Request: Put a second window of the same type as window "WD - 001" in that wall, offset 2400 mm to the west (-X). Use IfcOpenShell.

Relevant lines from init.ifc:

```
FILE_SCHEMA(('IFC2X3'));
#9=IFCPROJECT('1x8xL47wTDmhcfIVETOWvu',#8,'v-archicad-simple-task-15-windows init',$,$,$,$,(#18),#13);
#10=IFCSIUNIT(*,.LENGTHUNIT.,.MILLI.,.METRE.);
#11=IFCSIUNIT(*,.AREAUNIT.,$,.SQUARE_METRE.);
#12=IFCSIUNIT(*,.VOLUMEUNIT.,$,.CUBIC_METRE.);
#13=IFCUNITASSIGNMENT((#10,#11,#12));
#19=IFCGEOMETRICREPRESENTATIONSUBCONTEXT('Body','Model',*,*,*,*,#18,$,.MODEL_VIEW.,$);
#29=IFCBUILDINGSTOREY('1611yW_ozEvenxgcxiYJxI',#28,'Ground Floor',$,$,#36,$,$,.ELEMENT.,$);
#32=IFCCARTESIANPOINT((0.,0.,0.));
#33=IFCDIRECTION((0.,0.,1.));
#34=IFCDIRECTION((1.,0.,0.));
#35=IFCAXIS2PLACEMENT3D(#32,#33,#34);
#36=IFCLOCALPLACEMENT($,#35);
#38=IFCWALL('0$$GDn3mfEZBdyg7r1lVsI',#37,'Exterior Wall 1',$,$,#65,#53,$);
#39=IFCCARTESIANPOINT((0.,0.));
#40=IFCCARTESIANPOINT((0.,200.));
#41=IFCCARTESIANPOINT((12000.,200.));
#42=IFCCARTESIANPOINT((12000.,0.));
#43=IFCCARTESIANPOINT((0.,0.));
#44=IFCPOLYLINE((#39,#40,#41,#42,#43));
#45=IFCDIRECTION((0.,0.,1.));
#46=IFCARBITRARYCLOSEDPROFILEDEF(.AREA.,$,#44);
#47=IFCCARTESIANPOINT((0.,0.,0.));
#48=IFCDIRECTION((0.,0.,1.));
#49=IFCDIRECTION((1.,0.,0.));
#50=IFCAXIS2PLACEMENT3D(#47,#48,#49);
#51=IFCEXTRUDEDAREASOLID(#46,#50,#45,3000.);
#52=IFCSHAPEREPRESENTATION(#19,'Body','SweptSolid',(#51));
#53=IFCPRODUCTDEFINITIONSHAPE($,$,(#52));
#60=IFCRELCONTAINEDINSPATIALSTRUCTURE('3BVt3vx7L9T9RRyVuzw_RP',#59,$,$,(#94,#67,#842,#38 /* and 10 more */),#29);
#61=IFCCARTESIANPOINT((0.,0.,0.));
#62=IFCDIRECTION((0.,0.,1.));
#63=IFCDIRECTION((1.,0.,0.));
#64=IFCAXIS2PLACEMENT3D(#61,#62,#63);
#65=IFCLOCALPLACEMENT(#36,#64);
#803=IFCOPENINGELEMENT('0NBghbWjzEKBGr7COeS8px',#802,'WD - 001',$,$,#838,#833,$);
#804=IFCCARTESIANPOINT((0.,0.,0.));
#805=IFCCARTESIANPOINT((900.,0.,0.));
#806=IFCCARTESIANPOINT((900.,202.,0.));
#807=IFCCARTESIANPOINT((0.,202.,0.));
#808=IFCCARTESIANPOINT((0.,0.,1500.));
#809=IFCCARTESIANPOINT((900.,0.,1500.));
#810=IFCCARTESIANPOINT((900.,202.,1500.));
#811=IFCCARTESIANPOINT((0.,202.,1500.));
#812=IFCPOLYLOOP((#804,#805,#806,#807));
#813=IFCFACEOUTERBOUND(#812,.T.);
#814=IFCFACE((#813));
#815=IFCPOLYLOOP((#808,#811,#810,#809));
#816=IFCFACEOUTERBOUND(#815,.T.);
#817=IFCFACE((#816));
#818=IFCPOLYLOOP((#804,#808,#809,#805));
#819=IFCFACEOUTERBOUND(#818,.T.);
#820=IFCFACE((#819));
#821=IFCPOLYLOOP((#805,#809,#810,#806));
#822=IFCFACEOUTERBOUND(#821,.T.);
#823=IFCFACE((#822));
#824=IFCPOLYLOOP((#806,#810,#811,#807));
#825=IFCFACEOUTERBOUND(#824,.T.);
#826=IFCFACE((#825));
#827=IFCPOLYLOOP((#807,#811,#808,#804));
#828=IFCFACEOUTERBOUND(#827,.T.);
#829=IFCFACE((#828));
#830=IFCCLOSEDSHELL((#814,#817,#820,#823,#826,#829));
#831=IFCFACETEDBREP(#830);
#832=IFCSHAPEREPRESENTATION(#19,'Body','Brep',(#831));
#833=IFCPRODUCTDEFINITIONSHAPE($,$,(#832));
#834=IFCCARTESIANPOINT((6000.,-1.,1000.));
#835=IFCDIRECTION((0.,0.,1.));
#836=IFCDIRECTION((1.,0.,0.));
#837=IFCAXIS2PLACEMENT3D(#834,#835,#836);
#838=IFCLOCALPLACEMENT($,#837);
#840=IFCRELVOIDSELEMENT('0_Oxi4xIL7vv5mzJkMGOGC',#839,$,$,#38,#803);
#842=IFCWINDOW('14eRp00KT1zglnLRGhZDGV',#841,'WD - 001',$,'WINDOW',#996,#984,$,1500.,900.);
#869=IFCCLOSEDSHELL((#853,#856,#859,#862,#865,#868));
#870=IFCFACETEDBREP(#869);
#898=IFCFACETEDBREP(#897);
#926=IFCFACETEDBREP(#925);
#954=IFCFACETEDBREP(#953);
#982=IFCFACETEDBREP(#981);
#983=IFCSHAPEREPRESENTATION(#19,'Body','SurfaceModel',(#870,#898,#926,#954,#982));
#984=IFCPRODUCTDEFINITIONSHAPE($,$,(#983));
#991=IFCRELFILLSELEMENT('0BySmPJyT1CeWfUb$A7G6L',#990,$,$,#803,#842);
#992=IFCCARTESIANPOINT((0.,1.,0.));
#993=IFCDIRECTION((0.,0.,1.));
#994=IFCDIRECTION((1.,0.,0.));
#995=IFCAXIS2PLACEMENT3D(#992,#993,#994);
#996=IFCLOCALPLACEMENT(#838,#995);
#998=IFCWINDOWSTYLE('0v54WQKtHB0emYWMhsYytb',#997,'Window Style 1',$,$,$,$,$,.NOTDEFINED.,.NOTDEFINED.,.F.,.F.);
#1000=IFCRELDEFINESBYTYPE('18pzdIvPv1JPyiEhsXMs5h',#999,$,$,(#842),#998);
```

```python
import ifcopenshell
import ifcopenshell.api.feature
import ifcopenshell.api.geometry
import ifcopenshell.api.root
import ifcopenshell.geom
import ifcopenshell.util.element
import ifcopenshell.util.placement
import ifcopenshell.util.shape
import ifcopenshell.util.unit

model = ifcopenshell.open("init.ifc")
unit_scale = ifcopenshell.util.unit.calculate_unit_scale(model)
settings = ifcopenshell.geom.settings()


def volume(element):
    """Net volume in cubic metres, openings subtracted."""
    shape = ifcopenshell.geom.create_shape(settings, element)
    return ifcopenshell.util.shape.get_volume(shape.geometry)


window = model.by_guid("14eRp00KT1zglnLRGhZDGV")
opening = window.FillsVoids[0].RelatingOpeningElement
wall = opening.VoidsElements[0].RelatingBuildingElement
before = volume(wall)
shift = ifcopenshell.util.placement.get_local_placement(wall.ObjectPlacement)[:3, 0] * -2.4 / unit_scale

# copy_class copies the void relationship, type, container and properties, but no geometry.
new_opening = ifcopenshell.api.root.copy_class(model, product=opening)
new_opening.Representation = ifcopenshell.util.element.copy_deep(
    model, opening.Representation, exclude=["IfcGeometricRepresentationContext", "IfcRepresentationMap"]
)
new_window = ifcopenshell.api.root.copy_class(model, product=window)
new_window.Representation = ifcopenshell.util.element.copy_deep(
    model, window.Representation, exclude=["IfcGeometricRepresentationContext", "IfcRepresentationMap"]
)
fills = ifcopenshell.api.feature.add_filling(model, opening=new_opening, element=new_window)
fills.OwnerHistory = new_window.OwnerHistory  # required in IFC2X3

for old, new in ((opening, new_opening), (window, new_window)):
    matrix = ifcopenshell.util.placement.get_local_placement(old.ObjectPlacement)
    matrix[:3, 3] += shift
    ifcopenshell.api.geometry.edit_object_placement(model, product=new, matrix=matrix, is_si=False)

after = volume(wall)

print(f"wall volume {before:.3f} -> {after:.3f} m3")

model.write("init_rev.ifc")
```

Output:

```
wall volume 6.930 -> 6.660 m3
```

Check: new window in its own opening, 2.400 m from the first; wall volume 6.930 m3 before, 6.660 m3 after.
